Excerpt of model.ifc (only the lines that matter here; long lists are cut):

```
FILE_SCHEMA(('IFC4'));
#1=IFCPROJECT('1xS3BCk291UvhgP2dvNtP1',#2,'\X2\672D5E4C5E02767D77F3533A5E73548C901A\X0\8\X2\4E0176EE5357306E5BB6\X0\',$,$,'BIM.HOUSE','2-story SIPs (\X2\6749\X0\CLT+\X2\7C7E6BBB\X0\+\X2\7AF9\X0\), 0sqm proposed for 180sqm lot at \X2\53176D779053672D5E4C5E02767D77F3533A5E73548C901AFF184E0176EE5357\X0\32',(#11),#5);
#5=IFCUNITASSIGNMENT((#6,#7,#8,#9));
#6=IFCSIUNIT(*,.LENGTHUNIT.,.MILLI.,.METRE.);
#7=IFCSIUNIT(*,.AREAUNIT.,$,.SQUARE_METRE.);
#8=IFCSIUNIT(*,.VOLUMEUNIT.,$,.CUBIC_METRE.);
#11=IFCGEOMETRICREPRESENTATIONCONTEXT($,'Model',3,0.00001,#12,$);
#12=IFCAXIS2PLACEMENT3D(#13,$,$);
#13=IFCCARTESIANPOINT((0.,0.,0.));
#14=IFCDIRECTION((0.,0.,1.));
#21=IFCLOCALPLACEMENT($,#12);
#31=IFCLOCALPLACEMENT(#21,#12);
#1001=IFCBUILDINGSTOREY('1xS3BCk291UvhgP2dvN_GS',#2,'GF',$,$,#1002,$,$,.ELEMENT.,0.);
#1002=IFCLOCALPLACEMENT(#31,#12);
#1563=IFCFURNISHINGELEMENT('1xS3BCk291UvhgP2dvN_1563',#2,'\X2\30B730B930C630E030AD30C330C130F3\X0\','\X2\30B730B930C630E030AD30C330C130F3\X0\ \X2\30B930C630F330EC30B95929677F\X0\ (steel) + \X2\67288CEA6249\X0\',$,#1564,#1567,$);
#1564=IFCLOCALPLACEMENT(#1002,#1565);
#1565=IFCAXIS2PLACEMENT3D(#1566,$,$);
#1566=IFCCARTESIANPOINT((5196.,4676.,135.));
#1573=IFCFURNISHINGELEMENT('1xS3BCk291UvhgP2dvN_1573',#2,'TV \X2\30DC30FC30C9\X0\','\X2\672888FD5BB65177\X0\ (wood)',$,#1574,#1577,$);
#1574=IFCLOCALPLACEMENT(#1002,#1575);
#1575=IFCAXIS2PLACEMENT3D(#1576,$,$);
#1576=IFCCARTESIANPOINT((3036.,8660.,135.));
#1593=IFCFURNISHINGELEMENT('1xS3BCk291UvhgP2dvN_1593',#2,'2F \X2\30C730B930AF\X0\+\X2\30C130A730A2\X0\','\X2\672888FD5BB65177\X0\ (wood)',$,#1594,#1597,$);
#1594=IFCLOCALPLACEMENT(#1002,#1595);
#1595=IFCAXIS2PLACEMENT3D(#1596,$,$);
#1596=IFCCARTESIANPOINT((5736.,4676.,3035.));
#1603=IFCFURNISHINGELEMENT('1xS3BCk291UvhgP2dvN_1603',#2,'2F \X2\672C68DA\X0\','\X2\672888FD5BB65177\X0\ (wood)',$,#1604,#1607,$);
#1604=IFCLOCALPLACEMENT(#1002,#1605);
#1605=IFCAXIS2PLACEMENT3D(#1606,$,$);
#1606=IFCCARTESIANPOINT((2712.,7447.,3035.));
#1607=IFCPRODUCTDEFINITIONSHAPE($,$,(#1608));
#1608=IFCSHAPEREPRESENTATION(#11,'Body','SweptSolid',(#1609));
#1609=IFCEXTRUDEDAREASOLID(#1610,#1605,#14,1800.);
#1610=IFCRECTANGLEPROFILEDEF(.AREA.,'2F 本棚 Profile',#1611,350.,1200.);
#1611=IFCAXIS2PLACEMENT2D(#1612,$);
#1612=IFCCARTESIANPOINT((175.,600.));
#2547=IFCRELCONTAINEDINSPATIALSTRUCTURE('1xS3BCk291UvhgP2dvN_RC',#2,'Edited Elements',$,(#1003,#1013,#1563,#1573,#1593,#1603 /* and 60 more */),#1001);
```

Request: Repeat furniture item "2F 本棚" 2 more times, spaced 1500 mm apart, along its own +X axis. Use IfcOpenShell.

```python
import ifcopenshell
import ifcopenshell.api.geometry
import ifcopenshell.api.root
import ifcopenshell.util.element
import ifcopenshell.util.placement

model = ifcopenshell.open("model.ifc")


def reuse_history(source, copy):
    """copy_class also copies each property set's owner history, people and application; keep the originals."""
    for rel in copy.IsDefinedBy:
        if rel.is_a("IfcRelDefinesByProperties") and (history := rel.RelatingPropertyDefinition.OwnerHistory):
            rel.RelatingPropertyDefinition.OwnerHistory = source.OwnerHistory
            ifcopenshell.util.element.remove_deep2(model, history)


source = model.by_guid("1xS3BCk291UvhgP2dvN_1603")
base = ifcopenshell.util.placement.get_local_placement(source.ObjectPlacement)
step = base[:3, 0] * 1500.0

for i in range(1, 3):
    copy = ifcopenshell.api.root.copy_class(model, product=source)
    copy.Representation = ifcopenshell.util.element.copy_deep(
        model, source.Representation, exclude=["IfcGeometricRepresentationContext", "IfcRepresentationMap"]
    )
    reuse_history(source, copy)
    matrix = base.copy()
    matrix[:3, 3] += i * step
    print("added at", matrix[:3, 3].round(3) + 0.0)
    ifcopenshell.api.geometry.edit_object_placement(model, product=copy, matrix=matrix, is_si=False)

model.write("model-out.ifc")
```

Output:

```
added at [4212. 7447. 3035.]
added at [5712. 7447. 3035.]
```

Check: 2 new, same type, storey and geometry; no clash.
